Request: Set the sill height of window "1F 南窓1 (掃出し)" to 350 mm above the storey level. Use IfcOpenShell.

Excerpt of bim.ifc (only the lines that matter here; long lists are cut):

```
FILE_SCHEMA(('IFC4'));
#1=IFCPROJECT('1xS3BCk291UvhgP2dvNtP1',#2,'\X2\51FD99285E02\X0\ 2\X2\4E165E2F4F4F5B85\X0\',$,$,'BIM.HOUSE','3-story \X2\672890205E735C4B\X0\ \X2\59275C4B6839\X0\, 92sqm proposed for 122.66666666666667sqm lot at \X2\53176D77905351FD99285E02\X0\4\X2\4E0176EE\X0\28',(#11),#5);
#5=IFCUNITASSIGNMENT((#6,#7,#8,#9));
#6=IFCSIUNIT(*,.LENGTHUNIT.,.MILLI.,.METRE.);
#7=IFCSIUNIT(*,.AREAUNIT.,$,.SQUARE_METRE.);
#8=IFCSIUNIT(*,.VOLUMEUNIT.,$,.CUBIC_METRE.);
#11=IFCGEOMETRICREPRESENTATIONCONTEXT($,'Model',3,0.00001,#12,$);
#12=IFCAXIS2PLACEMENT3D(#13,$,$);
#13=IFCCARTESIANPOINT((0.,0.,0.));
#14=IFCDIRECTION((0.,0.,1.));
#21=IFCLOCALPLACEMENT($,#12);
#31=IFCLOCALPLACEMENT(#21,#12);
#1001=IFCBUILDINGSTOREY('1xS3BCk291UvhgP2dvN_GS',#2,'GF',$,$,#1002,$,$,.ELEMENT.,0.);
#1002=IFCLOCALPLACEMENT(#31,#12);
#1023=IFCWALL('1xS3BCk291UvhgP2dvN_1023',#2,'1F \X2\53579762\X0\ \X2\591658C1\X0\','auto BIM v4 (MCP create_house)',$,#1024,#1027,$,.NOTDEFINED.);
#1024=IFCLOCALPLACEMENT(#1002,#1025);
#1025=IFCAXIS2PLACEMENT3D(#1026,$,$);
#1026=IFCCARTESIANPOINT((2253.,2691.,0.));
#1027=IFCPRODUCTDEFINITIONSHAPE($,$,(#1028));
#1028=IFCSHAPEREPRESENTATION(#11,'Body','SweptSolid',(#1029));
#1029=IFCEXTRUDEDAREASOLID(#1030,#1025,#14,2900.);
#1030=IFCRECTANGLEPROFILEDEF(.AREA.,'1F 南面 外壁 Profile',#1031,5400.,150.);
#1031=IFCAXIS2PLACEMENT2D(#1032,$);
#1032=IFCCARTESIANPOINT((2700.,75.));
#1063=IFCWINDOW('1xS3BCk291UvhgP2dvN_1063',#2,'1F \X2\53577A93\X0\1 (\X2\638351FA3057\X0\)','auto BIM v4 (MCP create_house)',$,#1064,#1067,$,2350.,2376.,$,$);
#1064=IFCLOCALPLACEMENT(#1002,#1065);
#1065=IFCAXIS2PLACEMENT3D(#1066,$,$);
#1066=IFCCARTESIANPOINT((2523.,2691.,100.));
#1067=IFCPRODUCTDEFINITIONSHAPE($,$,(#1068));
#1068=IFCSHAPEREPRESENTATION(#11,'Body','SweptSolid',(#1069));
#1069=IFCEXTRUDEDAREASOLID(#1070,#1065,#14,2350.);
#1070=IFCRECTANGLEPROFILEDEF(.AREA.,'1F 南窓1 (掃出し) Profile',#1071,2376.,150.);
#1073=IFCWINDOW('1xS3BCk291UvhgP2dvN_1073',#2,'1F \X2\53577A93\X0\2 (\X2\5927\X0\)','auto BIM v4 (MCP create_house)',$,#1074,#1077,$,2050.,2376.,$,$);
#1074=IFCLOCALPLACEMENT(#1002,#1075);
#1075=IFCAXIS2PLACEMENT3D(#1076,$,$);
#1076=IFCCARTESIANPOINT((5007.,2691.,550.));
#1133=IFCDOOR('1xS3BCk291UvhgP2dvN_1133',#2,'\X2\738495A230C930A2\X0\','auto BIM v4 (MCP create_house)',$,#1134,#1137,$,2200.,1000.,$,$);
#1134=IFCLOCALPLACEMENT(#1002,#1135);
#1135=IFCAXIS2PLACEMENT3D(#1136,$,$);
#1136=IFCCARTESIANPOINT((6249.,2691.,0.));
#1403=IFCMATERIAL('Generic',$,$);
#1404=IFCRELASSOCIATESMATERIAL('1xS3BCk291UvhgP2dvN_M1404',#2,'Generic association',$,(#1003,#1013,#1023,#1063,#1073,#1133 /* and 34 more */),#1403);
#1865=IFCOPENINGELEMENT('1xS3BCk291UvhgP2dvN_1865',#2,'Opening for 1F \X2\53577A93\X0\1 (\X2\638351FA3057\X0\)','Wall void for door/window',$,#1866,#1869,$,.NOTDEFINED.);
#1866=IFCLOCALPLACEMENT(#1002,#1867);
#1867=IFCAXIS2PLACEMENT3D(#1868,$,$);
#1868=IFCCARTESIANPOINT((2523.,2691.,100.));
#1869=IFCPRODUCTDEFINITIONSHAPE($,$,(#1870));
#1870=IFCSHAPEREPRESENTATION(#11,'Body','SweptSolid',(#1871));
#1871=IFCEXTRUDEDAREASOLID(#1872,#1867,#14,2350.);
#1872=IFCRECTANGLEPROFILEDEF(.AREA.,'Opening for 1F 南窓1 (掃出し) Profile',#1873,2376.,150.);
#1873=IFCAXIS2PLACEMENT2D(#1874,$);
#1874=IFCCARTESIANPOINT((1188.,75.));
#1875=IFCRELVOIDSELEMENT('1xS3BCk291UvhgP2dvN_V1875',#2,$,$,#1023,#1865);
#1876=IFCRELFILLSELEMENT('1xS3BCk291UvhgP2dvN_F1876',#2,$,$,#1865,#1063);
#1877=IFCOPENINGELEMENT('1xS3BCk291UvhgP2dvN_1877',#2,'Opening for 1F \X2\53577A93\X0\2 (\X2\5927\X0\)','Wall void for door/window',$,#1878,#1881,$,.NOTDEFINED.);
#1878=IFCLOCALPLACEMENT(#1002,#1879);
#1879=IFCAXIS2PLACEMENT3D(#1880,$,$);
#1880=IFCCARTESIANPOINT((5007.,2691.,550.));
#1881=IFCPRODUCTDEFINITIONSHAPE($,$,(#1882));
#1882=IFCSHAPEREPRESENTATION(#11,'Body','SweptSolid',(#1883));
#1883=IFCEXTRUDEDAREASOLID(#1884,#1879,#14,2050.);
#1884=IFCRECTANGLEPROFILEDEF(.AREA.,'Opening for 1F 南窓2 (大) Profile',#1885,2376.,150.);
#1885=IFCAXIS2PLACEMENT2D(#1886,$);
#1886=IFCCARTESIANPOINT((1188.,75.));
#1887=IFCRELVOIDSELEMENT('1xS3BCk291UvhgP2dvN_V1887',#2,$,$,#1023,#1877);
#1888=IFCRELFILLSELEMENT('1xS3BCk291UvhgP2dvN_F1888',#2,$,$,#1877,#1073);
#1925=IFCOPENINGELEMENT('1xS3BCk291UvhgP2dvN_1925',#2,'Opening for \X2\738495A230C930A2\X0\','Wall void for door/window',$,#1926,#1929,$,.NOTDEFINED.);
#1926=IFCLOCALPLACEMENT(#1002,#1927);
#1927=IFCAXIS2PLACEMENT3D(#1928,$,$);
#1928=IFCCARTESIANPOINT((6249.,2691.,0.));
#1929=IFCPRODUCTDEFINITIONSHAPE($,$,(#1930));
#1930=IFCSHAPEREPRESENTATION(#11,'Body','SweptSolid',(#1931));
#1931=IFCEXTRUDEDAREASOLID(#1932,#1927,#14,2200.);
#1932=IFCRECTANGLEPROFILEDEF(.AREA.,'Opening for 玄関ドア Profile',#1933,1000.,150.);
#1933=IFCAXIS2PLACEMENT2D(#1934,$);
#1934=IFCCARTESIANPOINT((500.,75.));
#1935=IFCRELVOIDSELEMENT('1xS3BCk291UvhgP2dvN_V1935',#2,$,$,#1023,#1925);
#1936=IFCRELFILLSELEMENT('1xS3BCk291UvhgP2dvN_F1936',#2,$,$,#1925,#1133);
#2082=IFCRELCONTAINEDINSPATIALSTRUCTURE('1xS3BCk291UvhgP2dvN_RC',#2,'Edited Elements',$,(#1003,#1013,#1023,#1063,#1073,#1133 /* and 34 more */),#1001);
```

```python
import numpy as np
import ifcopenshell
import ifcopenshell.api.geometry
import ifcopenshell.geom
import ifcopenshell.util.element
import ifcopenshell.util.placement
import ifcopenshell.util.shape
import ifcopenshell.util.unit

model = ifcopenshell.open("bim.ifc")
unit_scale = ifcopenshell.util.unit.calculate_unit_scale(model)

window = model.by_id(1063)
opening = window.FillsVoids[0].RelatingOpeningElement
storey = ifcopenshell.util.element.get_container(window, ifc_class="IfcBuildingStorey")
level = ifcopenshell.util.placement.get_local_placement(storey.ObjectPlacement)[2, 3]

# The opening's origin need not be at the sill, so measure its lowest point.
shape = ifcopenshell.geom.create_shape(ifcopenshell.geom.settings(), opening)
bottom = ifcopenshell.util.shape.get_shape_bottom_elevation(shape, shape.geometry) / unit_scale
dz = level + 0.35 / unit_scale - bottom

shift = np.array([0.0, 0.0, dz])
# The window is not placed relative to its opening, so move both.
for product in (opening, window):
    matrix = ifcopenshell.util.placement.get_local_placement(product.ObjectPlacement)
    matrix[:3, 3] += shift
    ifcopenshell.api.geometry.edit_object_placement(model, product=product, matrix=matrix, is_si=False)

print(f"moved by {dz * unit_scale:+.3f} m")

model.write("bim_v2.ifc")
```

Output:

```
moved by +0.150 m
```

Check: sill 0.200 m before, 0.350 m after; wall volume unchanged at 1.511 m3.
